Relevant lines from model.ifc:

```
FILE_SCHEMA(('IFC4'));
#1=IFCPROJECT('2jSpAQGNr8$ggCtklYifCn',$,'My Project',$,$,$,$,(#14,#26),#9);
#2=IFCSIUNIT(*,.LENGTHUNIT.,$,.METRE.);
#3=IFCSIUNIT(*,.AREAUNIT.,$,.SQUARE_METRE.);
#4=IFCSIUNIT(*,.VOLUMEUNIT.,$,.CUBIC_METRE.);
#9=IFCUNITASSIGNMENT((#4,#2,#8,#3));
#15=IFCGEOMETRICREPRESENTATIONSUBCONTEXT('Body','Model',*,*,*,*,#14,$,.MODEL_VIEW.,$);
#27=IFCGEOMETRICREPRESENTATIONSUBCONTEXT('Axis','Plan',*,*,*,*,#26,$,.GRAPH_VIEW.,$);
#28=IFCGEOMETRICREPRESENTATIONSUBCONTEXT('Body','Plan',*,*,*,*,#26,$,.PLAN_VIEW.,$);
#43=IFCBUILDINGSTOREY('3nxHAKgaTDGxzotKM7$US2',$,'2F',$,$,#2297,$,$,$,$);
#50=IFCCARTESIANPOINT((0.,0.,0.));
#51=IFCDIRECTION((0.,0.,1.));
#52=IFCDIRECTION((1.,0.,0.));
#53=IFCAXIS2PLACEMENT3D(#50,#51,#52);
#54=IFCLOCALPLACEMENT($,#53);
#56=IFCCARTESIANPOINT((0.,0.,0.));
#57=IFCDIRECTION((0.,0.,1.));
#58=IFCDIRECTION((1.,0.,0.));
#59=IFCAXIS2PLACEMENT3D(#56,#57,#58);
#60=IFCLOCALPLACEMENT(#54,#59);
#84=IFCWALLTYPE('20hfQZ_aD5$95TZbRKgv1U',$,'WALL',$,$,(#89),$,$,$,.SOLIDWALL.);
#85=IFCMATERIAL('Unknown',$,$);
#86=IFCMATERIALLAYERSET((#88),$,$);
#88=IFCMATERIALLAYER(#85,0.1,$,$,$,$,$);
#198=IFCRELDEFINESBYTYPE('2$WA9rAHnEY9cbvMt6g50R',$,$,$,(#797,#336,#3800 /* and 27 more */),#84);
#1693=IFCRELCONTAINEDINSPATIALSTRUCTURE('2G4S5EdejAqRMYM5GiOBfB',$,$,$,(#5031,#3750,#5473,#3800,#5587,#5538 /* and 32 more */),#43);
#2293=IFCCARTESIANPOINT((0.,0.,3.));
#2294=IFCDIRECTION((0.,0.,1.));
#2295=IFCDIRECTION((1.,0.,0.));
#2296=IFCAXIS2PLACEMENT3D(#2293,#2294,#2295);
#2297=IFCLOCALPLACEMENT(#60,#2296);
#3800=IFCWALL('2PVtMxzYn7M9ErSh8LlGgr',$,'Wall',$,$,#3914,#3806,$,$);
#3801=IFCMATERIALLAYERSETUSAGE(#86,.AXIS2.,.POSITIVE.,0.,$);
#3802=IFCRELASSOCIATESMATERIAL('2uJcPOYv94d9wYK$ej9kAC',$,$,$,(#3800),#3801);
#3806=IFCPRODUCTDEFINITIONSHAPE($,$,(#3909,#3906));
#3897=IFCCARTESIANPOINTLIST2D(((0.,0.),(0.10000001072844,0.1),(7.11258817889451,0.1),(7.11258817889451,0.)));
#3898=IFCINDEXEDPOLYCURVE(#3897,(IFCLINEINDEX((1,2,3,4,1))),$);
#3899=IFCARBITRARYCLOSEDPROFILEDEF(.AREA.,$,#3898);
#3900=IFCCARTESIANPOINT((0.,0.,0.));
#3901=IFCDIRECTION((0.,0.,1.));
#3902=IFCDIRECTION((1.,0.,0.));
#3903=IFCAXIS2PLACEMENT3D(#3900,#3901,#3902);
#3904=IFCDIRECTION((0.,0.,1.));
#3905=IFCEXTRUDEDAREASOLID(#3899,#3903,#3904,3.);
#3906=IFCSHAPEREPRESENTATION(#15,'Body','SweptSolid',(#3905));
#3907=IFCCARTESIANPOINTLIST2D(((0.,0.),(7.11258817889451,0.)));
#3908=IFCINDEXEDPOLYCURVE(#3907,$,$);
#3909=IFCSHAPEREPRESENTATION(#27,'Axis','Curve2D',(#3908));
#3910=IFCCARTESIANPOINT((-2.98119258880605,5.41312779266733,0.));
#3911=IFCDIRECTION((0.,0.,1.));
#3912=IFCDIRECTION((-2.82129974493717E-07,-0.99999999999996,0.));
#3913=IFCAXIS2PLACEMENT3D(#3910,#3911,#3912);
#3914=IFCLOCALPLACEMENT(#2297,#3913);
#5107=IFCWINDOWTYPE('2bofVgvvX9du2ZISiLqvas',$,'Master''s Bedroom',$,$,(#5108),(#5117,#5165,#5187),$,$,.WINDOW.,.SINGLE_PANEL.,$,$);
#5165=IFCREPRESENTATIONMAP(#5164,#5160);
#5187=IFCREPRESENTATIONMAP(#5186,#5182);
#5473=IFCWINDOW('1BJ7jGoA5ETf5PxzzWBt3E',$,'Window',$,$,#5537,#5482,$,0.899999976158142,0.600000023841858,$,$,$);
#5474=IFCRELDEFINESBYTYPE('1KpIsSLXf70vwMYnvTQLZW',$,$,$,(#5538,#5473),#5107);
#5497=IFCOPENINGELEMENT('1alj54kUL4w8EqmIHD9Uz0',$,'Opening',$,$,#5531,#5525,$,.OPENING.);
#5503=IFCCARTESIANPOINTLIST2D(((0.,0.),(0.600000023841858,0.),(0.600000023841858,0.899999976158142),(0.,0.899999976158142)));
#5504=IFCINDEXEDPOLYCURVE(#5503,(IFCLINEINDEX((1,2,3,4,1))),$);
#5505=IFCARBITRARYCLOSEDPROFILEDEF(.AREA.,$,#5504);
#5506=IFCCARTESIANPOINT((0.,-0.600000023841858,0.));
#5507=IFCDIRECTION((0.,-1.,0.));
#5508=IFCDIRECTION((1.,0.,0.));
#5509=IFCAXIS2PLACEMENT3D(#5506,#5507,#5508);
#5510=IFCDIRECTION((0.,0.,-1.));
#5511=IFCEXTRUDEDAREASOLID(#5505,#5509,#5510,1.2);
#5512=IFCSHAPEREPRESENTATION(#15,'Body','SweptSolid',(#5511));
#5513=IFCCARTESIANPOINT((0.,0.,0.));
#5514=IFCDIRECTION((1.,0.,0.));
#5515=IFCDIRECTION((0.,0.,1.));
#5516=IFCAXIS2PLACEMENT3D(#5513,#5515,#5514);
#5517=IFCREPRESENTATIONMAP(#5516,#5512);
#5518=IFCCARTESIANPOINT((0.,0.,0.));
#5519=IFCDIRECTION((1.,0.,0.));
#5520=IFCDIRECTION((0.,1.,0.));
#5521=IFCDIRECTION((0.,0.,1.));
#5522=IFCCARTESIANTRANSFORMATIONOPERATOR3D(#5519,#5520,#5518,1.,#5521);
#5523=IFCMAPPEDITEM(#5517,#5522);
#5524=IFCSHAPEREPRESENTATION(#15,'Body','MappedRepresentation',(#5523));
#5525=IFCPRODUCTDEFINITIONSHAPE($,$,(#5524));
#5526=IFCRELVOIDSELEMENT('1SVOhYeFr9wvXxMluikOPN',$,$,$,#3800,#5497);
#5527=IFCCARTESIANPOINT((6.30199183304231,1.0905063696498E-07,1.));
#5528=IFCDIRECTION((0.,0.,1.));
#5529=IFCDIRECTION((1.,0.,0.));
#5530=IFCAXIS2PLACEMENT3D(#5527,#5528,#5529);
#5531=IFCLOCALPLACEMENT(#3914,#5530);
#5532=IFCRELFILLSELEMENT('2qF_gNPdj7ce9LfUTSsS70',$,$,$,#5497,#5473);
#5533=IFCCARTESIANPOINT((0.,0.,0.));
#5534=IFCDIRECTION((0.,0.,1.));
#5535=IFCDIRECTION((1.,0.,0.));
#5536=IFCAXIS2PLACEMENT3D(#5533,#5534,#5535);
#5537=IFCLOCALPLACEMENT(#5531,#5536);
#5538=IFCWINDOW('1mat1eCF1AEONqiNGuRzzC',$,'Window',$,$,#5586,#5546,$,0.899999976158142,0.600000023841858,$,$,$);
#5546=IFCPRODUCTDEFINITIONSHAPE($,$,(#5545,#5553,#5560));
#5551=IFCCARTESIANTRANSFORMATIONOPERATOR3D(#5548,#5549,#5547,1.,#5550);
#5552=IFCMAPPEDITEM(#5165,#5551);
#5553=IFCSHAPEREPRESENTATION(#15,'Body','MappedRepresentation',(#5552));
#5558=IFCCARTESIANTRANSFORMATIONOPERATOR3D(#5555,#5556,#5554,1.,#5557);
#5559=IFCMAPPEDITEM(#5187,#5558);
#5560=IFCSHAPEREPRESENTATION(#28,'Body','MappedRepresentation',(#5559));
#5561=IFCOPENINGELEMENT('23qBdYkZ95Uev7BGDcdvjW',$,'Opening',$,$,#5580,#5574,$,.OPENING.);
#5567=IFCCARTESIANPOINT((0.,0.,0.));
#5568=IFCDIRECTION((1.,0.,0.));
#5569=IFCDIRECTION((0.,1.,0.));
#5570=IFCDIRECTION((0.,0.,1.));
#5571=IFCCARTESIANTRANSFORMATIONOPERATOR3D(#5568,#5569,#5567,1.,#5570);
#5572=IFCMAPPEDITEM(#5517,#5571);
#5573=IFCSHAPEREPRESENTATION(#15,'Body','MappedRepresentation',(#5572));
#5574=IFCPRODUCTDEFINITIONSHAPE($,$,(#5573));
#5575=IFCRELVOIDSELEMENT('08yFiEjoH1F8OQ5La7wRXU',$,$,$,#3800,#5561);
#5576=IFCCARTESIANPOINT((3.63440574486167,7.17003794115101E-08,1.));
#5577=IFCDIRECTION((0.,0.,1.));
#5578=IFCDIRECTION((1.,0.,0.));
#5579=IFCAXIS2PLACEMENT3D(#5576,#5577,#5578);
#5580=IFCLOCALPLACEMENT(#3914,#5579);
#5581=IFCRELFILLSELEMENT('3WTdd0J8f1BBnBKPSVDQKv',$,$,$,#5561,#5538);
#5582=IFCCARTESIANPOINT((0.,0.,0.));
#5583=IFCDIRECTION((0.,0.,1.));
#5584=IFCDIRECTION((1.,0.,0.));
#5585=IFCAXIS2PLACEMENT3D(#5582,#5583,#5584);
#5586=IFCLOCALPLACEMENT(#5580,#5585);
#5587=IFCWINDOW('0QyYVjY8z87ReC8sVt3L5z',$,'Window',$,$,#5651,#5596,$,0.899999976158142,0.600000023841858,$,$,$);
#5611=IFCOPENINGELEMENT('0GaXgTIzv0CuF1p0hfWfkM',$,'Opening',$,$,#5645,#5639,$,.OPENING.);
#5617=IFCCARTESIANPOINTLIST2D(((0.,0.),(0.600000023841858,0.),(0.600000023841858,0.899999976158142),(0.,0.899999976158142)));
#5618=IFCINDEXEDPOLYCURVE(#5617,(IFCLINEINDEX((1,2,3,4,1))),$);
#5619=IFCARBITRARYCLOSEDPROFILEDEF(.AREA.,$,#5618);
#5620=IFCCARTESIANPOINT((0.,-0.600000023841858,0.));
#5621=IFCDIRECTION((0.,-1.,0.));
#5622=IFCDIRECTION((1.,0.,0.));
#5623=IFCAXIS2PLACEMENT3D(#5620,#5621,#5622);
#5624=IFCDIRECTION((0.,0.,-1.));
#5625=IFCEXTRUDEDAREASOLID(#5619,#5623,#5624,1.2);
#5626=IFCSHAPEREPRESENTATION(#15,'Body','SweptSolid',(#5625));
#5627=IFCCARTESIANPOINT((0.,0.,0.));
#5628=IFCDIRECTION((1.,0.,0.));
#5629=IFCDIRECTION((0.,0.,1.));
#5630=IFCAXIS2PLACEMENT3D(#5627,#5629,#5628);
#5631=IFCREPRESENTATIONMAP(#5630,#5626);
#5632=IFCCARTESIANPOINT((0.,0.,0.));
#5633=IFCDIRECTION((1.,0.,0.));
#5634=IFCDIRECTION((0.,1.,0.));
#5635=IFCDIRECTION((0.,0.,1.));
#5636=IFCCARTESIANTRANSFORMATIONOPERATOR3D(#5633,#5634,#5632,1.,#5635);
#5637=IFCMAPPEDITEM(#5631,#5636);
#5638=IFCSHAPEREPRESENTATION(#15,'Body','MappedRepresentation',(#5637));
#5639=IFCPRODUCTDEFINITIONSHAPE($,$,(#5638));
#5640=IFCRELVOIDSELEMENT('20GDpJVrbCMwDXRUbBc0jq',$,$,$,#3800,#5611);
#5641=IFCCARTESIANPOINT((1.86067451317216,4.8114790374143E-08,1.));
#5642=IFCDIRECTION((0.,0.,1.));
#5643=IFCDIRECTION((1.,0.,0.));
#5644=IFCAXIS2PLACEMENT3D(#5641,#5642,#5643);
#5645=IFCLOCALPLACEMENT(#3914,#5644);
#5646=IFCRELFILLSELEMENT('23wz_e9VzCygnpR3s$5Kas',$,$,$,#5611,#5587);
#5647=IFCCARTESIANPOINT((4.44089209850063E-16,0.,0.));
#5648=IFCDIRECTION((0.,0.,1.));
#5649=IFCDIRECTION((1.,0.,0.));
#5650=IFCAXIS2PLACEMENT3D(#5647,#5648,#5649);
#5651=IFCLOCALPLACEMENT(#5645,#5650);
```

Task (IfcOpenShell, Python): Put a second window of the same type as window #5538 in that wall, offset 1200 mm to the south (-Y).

```python
import ifcopenshell
import ifcopenshell.api.feature
import ifcopenshell.api.geometry
import ifcopenshell.api.root
import ifcopenshell.geom
import ifcopenshell.util.element
import ifcopenshell.util.placement
import ifcopenshell.util.shape
import ifcopenshell.util.unit

model = ifcopenshell.open("model.ifc")
unit_scale = ifcopenshell.util.unit.calculate_unit_scale(model)
settings = ifcopenshell.geom.settings()


def volume(element):
    """Net volume in cubic metres, openings subtracted."""
    shape = ifcopenshell.geom.create_shape(settings, element)
    return ifcopenshell.util.shape.get_volume(shape.geometry)


window = model.by_guid("1mat1eCF1AEONqiNGuRzzC")
opening = window.FillsVoids[0].RelatingOpeningElement
wall = opening.VoidsElements[0].RelatingBuildingElement
before = volume(wall)
shift = ifcopenshell.util.placement.get_local_placement(wall.ObjectPlacement)[:3, 0] * 1.2 / unit_scale

# copy_class copies the void relationship, type, container and properties, but no geometry.
new_opening = ifcopenshell.api.root.copy_class(model, product=opening)
new_opening.Representation = ifcopenshell.util.element.copy_deep(
    model, opening.Representation, exclude=["IfcGeometricRepresentationContext", "IfcRepresentationMap"]
)
new_window = ifcopenshell.api.root.copy_class(model, product=window)
new_window.Representation = ifcopenshell.util.element.copy_deep(
    model, window.Representation, exclude=["IfcGeometricRepresentationContext", "IfcRepresentationMap"]
)
ifcopenshell.api.feature.add_filling(model, opening=new_opening, element=new_window)

for old, new in ((opening, new_opening), (window, new_window)):
    matrix = ifcopenshell.util.placement.get_local_placement(old.ObjectPlacement)
    matrix[:3, 3] += shift
    ifcopenshell.api.geometry.edit_object_placement(model, product=new, matrix=matrix, is_si=False)

after = volume(wall)

print(f"wall volume {before:.3f} -> {after:.3f} m3")

model.write("model_v2.ifc")
```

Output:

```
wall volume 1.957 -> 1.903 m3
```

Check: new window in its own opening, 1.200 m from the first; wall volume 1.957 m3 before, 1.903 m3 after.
